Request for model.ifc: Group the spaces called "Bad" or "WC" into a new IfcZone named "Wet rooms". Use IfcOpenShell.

First a look at what the model holds.

```python
import ifcopenshell

model = ifcopenshell.open("model.ifc")
print(model.schema)
seen = {}
for space in model.by_type("IfcSpace"):
    seen[space.LongName] = seen.get(space.LongName, 0) + 1
for name, count in sorted(seen.items(), key=str):
    print(count, "x", name)
print("zones:", [z.Name for z in model.by_type("IfcZone")][:20])
```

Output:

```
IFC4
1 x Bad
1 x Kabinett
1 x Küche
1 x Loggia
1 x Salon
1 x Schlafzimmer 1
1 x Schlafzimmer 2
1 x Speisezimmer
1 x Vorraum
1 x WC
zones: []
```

```python
import ifcopenshell
import ifcopenshell.api.group
import ifcopenshell.api.root

model = ifcopenshell.open("model.ifc")

names = {"Bad", "WC"}
spaces = [s for s in model.by_type("IfcSpace") if s.LongName in names]

zone = ifcopenshell.api.root.create_entity(model, ifc_class="IfcZone", name="Wet rooms")
ifcopenshell.api.group.assign_group(model, products=spaces, group=zone)
print(len(spaces), "spaces in", zone.Name)

model.write("model-out.ifc")
```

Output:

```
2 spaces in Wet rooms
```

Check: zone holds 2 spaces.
